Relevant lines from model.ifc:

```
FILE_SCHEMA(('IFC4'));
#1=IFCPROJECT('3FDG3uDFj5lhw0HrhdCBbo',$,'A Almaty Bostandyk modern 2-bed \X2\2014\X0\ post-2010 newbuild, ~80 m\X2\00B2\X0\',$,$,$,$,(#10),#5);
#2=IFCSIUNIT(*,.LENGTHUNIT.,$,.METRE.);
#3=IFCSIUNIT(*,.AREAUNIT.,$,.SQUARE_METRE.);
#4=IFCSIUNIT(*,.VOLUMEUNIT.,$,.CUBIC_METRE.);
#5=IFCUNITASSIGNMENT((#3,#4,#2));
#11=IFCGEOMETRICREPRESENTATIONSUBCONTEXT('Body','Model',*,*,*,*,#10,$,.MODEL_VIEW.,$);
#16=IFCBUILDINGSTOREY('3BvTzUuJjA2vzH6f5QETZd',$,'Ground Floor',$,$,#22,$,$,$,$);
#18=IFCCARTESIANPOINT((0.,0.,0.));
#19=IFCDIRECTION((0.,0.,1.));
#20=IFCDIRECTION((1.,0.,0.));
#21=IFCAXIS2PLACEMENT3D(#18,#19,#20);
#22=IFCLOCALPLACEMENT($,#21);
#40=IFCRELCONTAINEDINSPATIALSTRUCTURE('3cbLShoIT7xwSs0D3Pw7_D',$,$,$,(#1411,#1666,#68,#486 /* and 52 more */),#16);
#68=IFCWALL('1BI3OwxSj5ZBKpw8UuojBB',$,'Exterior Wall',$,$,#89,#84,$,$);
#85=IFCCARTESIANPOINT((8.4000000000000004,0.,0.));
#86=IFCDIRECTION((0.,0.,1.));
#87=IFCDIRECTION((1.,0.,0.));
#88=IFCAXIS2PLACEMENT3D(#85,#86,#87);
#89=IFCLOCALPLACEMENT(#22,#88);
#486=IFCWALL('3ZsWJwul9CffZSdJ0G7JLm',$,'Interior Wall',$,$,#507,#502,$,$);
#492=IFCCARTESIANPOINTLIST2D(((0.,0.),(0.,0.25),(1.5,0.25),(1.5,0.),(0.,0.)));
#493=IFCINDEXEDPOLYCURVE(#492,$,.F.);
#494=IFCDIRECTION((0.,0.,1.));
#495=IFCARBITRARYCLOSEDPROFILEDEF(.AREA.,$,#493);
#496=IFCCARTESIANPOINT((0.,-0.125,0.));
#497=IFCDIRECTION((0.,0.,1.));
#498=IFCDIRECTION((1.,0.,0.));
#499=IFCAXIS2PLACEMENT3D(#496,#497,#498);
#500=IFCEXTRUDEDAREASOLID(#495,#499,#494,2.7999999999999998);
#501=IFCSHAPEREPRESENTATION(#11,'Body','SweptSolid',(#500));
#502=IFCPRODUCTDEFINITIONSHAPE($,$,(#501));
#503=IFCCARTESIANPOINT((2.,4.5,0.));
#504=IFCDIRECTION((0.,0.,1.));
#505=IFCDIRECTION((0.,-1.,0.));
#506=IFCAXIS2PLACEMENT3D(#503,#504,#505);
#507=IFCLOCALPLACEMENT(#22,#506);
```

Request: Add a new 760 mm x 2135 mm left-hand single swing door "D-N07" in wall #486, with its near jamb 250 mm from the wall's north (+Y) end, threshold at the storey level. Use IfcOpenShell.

```python
import numpy as np
import ifcopenshell
import ifcopenshell.api.feature
import ifcopenshell.api.geometry
import ifcopenshell.api.root
import ifcopenshell.api.spatial
import ifcopenshell.geom
import ifcopenshell.util.element
import ifcopenshell.util.placement
import ifcopenshell.util.representation
import ifcopenshell.util.shape
import ifcopenshell.util.unit

model = ifcopenshell.open("model.ifc")
unit_scale = ifcopenshell.util.unit.calculate_unit_scale(model)
settings = ifcopenshell.geom.settings()


def volume(element):
    """Net volume in cubic metres, openings subtracted."""
    shape = ifcopenshell.geom.create_shape(settings, element)
    return ifcopenshell.util.shape.get_volume(shape.geometry)


wall = model.by_guid("3ZsWJwul9CffZSdJ0G7JLm")
storey = ifcopenshell.util.element.get_container(wall, ifc_class="IfcBuildingStorey")
context = ifcopenshell.util.representation.get_context(model, "Model", "Body", "MODEL_VIEW")
before = volume(wall)

width, height, from_end, sill = 0.76, 2.135, 0.25, 0.0  # metres

# The wall runs along its own X axis, and the end named is its -X end.
wall_shape = ifcopenshell.geom.create_shape(settings, wall)
x, y, z = ifcopenshell.util.shape.get_vertices(wall_shape.geometry).T
start = x.min() + from_end
face, thickness = float(y.min()), float(y.max() - y.min())
wall_matrix = ifcopenshell.util.placement.get_local_placement(wall.ObjectPlacement)
level = ifcopenshell.util.placement.get_local_placement(storey.ObjectPlacement)[2, 3]


def in_wall(x, y):
    """Placement at x, y metres in the wall's axes, at sill height."""
    matrix = wall_matrix.copy()
    matrix[:, 3] = wall_matrix @ np.array([x / unit_scale, y / unit_scale, 0.0, 1.0])
    matrix[2, 3] = level + sill / unit_scale
    return matrix


# Opening: a box that overshoots both wall faces by 50 mm.
opening = ifcopenshell.api.root.create_entity(model, ifc_class="IfcOpeningElement", predefined_type="OPENING")
box = ifcopenshell.api.geometry.add_wall_representation(
    model, context=context, length=width, height=height, thickness=thickness + 0.1
)
ifcopenshell.api.geometry.assign_representation(model, product=opening, representation=box)
ifcopenshell.api.geometry.edit_object_placement(model, product=opening, matrix=in_wall(start, face - 0.05), is_si=False)
ifcopenshell.api.feature.add_feature(model, feature=opening, element=wall)

door = ifcopenshell.api.root.create_entity(model, ifc_class="IfcDoor", name="D-N07", predefined_type="DOOR")
door.OverallWidth, door.OverallHeight = width / unit_scale, height / unit_scale
door.OperationType = "SINGLE_SWING_LEFT"
body = ifcopenshell.api.geometry.add_door_representation(
    model,
    context=context,
    overall_width=door.OverallWidth,
    overall_height=door.OverallHeight,
    operation_type="SINGLE_SWING_LEFT",
    lining_properties={"LiningDepth": thickness / unit_scale, "ThresholdDepth": thickness / unit_scale},
)
ifcopenshell.api.geometry.assign_representation(model, product=door, representation=body)
ifcopenshell.api.spatial.assign_container(model, products=[door], relating_structure=storey)
ifcopenshell.api.feature.add_filling(model, opening=opening, element=door)

# The lining spans the wall, so the door starts at the wall face.
ifcopenshell.api.geometry.edit_object_placement(model, product=door, matrix=in_wall(start, face), is_si=False)

after = volume(wall)

print(f"wall volume {before:.3f} -> {after:.3f} m3")

model.write("model_v2.ifc")
```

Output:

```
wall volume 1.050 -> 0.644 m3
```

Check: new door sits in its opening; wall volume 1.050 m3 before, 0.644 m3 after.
